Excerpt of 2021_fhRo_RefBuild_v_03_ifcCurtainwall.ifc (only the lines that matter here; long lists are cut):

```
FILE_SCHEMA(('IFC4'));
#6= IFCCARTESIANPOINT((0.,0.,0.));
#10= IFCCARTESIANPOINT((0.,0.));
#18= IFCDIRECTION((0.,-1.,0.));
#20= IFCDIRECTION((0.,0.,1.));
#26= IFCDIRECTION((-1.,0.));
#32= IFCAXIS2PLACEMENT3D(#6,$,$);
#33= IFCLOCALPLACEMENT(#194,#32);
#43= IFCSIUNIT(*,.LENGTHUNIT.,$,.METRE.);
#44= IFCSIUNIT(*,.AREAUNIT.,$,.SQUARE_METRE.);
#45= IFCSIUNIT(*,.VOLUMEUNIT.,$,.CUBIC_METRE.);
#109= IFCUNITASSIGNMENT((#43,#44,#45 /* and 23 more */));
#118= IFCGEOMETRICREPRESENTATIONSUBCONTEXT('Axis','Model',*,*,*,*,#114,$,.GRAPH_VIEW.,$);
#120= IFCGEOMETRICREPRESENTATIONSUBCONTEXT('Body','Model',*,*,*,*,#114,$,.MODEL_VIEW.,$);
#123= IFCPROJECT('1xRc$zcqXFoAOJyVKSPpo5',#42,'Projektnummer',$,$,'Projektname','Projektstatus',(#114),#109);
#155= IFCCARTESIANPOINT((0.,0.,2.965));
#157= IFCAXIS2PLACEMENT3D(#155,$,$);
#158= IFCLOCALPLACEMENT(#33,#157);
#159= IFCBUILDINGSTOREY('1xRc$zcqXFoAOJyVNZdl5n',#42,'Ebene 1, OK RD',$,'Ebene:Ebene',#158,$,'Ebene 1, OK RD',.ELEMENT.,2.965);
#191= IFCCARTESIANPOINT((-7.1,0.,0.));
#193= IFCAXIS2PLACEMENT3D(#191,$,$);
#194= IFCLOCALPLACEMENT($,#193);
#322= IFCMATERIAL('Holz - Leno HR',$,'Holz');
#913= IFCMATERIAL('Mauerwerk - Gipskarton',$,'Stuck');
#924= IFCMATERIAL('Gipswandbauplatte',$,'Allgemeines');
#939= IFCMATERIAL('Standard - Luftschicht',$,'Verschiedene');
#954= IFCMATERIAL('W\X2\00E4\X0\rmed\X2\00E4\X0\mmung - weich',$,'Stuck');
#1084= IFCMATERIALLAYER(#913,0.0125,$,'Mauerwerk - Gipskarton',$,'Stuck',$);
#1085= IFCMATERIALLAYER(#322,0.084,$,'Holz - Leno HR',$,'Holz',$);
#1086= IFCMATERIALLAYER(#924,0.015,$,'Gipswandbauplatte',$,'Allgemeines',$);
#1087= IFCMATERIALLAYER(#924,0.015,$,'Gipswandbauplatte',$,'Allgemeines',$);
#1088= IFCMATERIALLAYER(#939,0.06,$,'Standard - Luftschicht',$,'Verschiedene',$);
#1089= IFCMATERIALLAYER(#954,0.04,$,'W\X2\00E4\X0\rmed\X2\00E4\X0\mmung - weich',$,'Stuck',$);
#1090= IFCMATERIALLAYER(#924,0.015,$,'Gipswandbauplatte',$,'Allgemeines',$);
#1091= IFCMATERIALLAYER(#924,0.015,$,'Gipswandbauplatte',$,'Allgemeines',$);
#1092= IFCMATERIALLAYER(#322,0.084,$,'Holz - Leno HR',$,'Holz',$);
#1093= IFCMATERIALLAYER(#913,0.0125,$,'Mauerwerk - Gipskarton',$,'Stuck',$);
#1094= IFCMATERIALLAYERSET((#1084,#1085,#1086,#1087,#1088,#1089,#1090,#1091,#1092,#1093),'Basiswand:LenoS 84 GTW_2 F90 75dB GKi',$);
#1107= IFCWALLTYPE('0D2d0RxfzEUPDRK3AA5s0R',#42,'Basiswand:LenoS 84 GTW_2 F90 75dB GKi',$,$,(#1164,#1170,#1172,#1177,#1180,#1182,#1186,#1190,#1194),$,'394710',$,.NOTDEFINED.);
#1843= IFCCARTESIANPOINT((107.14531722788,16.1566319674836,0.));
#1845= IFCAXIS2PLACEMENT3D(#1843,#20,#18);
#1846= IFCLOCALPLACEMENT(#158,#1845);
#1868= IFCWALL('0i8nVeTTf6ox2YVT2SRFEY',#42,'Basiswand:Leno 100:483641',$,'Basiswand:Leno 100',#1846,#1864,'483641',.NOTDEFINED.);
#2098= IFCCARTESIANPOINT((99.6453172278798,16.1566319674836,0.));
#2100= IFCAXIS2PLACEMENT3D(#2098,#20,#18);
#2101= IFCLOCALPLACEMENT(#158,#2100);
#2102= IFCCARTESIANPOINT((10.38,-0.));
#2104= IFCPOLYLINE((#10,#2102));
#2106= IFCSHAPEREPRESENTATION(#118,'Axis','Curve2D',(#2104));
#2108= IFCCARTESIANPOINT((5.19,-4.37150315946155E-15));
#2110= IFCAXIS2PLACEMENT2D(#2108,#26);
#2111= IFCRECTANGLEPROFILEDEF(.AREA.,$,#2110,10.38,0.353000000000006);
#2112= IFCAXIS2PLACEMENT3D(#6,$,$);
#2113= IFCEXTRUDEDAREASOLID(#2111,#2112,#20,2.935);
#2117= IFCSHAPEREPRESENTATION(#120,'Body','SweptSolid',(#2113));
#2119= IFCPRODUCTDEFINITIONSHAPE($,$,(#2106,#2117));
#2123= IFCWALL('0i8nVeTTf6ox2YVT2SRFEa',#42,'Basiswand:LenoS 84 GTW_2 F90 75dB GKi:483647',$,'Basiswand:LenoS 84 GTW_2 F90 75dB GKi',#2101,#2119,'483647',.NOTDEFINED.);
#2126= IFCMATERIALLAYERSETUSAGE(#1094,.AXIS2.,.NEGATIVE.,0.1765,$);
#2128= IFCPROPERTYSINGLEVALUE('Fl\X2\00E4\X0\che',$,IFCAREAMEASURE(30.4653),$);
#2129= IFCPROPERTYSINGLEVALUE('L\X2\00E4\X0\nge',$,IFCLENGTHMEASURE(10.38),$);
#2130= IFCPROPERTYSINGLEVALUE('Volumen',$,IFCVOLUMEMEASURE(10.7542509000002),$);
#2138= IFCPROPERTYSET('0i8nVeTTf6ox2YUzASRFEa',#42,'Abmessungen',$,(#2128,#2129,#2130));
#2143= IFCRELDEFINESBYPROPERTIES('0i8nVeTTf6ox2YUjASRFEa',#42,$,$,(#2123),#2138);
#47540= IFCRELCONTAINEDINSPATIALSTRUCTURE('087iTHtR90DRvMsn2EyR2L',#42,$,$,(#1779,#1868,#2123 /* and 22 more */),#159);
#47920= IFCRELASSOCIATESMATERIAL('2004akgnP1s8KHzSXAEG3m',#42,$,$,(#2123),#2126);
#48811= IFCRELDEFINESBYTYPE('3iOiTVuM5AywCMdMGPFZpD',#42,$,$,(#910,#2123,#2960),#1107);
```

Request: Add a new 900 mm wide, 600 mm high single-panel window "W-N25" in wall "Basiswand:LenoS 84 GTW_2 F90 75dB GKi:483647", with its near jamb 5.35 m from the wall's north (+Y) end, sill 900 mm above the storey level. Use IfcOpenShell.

```python
import numpy as np
import ifcopenshell
import ifcopenshell.api.feature
import ifcopenshell.api.geometry
import ifcopenshell.api.pset
import ifcopenshell.api.root
import ifcopenshell.api.spatial
import ifcopenshell.geom
import ifcopenshell.util.element
import ifcopenshell.util.placement
import ifcopenshell.util.representation
import ifcopenshell.util.shape
import ifcopenshell.util.unit

model = ifcopenshell.open("2021_fhRo_RefBuild_v_03_ifcCurtainwall.ifc")
unit_scale = ifcopenshell.util.unit.calculate_unit_scale(model)
area_scale = ifcopenshell.util.unit.calculate_unit_scale(model, "AREAUNIT")
volume_scale = ifcopenshell.util.unit.calculate_unit_scale(model, "VOLUMEUNIT")
settings = ifcopenshell.geom.settings()


def volume(element):
    """Net volume in cubic metres, openings subtracted."""
    shape = ifcopenshell.geom.create_shape(settings, element)
    return ifcopenshell.util.shape.get_volume(shape.geometry)


wall = model.by_guid("0i8nVeTTf6ox2YVT2SRFEa")
storey = ifcopenshell.util.element.get_container(wall, ifc_class="IfcBuildingStorey")
context = ifcopenshell.util.representation.get_context(model, "Model", "Body", "MODEL_VIEW")
before = volume(wall)

width, height, from_end, sill = 0.9, 0.6, 5.35, 0.9  # metres

# The wall runs along its own X axis, and the end named is its -X end.
wall_shape = ifcopenshell.geom.create_shape(settings, wall)
x, y, z = ifcopenshell.util.shape.get_vertices(wall_shape.geometry).T
start = x.min() + from_end
face, thickness = float(y.min()), float(y.max() - y.min())
wall_matrix = ifcopenshell.util.placement.get_local_placement(wall.ObjectPlacement)
level = ifcopenshell.util.placement.get_local_placement(storey.ObjectPlacement)[2, 3]


def in_wall(x, y):
    """Placement at x, y metres in the wall's axes, at sill height."""
    matrix = wall_matrix.copy()
    matrix[:, 3] = wall_matrix @ np.array([x / unit_scale, y / unit_scale, 0.0, 1.0])
    matrix[2, 3] = level + sill / unit_scale
    return matrix


# Opening: a box that overshoots both wall faces by 50 mm.
opening = ifcopenshell.api.root.create_entity(model, ifc_class="IfcOpeningElement", predefined_type="OPENING")
box = ifcopenshell.api.geometry.add_wall_representation(
    model, context=context, length=width, height=height, thickness=thickness + 0.1
)
ifcopenshell.api.geometry.assign_representation(model, product=opening, representation=box)
ifcopenshell.api.geometry.edit_object_placement(model, product=opening, matrix=in_wall(start, face - 0.05), is_si=False)
ifcopenshell.api.feature.add_feature(model, feature=opening, element=wall)

window = ifcopenshell.api.root.create_entity(model, ifc_class="IfcWindow", name="W-N25", predefined_type="WINDOW")
window.OverallWidth, window.OverallHeight = width / unit_scale, height / unit_scale
window.PartitioningType = "SINGLE_PANEL"
body = ifcopenshell.api.geometry.add_window_representation(
    model,
    context=context,
    overall_width=window.OverallWidth,
    overall_height=window.OverallHeight,
    partition_type="SINGLE_PANEL",
)
ifcopenshell.api.geometry.assign_representation(model, product=window, representation=body)
ifcopenshell.api.spatial.assign_container(model, products=[window], relating_structure=storey)
ifcopenshell.api.feature.add_filling(model, opening=opening, element=window)

# Centre the window in the wall's thickness.
ifcopenshell.api.geometry.edit_object_placement(model, product=window, matrix=in_wall(start, face), is_si=False)
window_shape = ifcopenshell.geom.create_shape(settings, window)
depth = ifcopenshell.util.shape.get_vertices(window_shape.geometry)[:, 1]
offset = face + thickness / 2 - (depth.min() + depth.max()) / 2
ifcopenshell.api.geometry.edit_object_placement(model, product=window, matrix=in_wall(start, offset), is_si=False)

after = volume(wall)

# Update the wall's stored quantities.
pset = model.by_id(ifcopenshell.util.element.get_pset(wall, "Abmessungen", should_inherit=False)["id"])
ifcopenshell.api.pset.edit_pset(model, pset=pset, properties={
    "Fläche": model.create_entity("IfcAreaMeasure", after / thickness / area_scale),
    "Volumen": model.create_entity("IfcVolumeMeasure", after / volume_scale),
})

print(f"wall volume {before:.3f} -> {after:.3f} m3")

model.write("2021_fhRo_RefBuild_v_03_ifcCurtainwall-out.ifc")
```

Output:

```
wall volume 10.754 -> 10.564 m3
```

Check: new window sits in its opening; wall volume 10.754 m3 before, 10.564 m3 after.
